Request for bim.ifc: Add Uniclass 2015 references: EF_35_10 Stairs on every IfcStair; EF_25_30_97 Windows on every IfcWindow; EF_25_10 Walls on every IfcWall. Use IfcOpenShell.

First a look at what the model holds.

```python
import ifcopenshell

model = ifcopenshell.open("bim.ifc")
print(model.schema)
print("classifications:", [c.Name for c in model.by_type("IfcClassification")])
for ifc_class in ("IfcDoor", "IfcRoof", "IfcStair", "IfcWall", "IfcWindow"):
    print(ifc_class, len(model.by_type(ifc_class)))
```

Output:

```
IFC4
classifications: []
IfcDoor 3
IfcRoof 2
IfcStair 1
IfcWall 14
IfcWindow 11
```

```python
import ifcopenshell
import ifcopenshell.api.classification

model = ifcopenshell.open("bim.ifc")

system = ifcopenshell.api.classification.add_classification(model, classification="Uniclass 2015")

codes = {
    "IfcStair": ("EF_35_10", "Stairs"),
    "IfcWindow": ("EF_25_30_97", "Windows"),
    "IfcWall": ("EF_25_10", "Walls"),
}
for ifc_class, (code, name) in codes.items():
    products = model.by_type(ifc_class)
    ifcopenshell.api.classification.add_reference(
        model, products=products, classification=system, identification=code, name=name
    )
    print(code, len(products))

model.write("bim_updated.ifc")
```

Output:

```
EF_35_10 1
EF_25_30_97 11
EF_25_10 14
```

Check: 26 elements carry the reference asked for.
